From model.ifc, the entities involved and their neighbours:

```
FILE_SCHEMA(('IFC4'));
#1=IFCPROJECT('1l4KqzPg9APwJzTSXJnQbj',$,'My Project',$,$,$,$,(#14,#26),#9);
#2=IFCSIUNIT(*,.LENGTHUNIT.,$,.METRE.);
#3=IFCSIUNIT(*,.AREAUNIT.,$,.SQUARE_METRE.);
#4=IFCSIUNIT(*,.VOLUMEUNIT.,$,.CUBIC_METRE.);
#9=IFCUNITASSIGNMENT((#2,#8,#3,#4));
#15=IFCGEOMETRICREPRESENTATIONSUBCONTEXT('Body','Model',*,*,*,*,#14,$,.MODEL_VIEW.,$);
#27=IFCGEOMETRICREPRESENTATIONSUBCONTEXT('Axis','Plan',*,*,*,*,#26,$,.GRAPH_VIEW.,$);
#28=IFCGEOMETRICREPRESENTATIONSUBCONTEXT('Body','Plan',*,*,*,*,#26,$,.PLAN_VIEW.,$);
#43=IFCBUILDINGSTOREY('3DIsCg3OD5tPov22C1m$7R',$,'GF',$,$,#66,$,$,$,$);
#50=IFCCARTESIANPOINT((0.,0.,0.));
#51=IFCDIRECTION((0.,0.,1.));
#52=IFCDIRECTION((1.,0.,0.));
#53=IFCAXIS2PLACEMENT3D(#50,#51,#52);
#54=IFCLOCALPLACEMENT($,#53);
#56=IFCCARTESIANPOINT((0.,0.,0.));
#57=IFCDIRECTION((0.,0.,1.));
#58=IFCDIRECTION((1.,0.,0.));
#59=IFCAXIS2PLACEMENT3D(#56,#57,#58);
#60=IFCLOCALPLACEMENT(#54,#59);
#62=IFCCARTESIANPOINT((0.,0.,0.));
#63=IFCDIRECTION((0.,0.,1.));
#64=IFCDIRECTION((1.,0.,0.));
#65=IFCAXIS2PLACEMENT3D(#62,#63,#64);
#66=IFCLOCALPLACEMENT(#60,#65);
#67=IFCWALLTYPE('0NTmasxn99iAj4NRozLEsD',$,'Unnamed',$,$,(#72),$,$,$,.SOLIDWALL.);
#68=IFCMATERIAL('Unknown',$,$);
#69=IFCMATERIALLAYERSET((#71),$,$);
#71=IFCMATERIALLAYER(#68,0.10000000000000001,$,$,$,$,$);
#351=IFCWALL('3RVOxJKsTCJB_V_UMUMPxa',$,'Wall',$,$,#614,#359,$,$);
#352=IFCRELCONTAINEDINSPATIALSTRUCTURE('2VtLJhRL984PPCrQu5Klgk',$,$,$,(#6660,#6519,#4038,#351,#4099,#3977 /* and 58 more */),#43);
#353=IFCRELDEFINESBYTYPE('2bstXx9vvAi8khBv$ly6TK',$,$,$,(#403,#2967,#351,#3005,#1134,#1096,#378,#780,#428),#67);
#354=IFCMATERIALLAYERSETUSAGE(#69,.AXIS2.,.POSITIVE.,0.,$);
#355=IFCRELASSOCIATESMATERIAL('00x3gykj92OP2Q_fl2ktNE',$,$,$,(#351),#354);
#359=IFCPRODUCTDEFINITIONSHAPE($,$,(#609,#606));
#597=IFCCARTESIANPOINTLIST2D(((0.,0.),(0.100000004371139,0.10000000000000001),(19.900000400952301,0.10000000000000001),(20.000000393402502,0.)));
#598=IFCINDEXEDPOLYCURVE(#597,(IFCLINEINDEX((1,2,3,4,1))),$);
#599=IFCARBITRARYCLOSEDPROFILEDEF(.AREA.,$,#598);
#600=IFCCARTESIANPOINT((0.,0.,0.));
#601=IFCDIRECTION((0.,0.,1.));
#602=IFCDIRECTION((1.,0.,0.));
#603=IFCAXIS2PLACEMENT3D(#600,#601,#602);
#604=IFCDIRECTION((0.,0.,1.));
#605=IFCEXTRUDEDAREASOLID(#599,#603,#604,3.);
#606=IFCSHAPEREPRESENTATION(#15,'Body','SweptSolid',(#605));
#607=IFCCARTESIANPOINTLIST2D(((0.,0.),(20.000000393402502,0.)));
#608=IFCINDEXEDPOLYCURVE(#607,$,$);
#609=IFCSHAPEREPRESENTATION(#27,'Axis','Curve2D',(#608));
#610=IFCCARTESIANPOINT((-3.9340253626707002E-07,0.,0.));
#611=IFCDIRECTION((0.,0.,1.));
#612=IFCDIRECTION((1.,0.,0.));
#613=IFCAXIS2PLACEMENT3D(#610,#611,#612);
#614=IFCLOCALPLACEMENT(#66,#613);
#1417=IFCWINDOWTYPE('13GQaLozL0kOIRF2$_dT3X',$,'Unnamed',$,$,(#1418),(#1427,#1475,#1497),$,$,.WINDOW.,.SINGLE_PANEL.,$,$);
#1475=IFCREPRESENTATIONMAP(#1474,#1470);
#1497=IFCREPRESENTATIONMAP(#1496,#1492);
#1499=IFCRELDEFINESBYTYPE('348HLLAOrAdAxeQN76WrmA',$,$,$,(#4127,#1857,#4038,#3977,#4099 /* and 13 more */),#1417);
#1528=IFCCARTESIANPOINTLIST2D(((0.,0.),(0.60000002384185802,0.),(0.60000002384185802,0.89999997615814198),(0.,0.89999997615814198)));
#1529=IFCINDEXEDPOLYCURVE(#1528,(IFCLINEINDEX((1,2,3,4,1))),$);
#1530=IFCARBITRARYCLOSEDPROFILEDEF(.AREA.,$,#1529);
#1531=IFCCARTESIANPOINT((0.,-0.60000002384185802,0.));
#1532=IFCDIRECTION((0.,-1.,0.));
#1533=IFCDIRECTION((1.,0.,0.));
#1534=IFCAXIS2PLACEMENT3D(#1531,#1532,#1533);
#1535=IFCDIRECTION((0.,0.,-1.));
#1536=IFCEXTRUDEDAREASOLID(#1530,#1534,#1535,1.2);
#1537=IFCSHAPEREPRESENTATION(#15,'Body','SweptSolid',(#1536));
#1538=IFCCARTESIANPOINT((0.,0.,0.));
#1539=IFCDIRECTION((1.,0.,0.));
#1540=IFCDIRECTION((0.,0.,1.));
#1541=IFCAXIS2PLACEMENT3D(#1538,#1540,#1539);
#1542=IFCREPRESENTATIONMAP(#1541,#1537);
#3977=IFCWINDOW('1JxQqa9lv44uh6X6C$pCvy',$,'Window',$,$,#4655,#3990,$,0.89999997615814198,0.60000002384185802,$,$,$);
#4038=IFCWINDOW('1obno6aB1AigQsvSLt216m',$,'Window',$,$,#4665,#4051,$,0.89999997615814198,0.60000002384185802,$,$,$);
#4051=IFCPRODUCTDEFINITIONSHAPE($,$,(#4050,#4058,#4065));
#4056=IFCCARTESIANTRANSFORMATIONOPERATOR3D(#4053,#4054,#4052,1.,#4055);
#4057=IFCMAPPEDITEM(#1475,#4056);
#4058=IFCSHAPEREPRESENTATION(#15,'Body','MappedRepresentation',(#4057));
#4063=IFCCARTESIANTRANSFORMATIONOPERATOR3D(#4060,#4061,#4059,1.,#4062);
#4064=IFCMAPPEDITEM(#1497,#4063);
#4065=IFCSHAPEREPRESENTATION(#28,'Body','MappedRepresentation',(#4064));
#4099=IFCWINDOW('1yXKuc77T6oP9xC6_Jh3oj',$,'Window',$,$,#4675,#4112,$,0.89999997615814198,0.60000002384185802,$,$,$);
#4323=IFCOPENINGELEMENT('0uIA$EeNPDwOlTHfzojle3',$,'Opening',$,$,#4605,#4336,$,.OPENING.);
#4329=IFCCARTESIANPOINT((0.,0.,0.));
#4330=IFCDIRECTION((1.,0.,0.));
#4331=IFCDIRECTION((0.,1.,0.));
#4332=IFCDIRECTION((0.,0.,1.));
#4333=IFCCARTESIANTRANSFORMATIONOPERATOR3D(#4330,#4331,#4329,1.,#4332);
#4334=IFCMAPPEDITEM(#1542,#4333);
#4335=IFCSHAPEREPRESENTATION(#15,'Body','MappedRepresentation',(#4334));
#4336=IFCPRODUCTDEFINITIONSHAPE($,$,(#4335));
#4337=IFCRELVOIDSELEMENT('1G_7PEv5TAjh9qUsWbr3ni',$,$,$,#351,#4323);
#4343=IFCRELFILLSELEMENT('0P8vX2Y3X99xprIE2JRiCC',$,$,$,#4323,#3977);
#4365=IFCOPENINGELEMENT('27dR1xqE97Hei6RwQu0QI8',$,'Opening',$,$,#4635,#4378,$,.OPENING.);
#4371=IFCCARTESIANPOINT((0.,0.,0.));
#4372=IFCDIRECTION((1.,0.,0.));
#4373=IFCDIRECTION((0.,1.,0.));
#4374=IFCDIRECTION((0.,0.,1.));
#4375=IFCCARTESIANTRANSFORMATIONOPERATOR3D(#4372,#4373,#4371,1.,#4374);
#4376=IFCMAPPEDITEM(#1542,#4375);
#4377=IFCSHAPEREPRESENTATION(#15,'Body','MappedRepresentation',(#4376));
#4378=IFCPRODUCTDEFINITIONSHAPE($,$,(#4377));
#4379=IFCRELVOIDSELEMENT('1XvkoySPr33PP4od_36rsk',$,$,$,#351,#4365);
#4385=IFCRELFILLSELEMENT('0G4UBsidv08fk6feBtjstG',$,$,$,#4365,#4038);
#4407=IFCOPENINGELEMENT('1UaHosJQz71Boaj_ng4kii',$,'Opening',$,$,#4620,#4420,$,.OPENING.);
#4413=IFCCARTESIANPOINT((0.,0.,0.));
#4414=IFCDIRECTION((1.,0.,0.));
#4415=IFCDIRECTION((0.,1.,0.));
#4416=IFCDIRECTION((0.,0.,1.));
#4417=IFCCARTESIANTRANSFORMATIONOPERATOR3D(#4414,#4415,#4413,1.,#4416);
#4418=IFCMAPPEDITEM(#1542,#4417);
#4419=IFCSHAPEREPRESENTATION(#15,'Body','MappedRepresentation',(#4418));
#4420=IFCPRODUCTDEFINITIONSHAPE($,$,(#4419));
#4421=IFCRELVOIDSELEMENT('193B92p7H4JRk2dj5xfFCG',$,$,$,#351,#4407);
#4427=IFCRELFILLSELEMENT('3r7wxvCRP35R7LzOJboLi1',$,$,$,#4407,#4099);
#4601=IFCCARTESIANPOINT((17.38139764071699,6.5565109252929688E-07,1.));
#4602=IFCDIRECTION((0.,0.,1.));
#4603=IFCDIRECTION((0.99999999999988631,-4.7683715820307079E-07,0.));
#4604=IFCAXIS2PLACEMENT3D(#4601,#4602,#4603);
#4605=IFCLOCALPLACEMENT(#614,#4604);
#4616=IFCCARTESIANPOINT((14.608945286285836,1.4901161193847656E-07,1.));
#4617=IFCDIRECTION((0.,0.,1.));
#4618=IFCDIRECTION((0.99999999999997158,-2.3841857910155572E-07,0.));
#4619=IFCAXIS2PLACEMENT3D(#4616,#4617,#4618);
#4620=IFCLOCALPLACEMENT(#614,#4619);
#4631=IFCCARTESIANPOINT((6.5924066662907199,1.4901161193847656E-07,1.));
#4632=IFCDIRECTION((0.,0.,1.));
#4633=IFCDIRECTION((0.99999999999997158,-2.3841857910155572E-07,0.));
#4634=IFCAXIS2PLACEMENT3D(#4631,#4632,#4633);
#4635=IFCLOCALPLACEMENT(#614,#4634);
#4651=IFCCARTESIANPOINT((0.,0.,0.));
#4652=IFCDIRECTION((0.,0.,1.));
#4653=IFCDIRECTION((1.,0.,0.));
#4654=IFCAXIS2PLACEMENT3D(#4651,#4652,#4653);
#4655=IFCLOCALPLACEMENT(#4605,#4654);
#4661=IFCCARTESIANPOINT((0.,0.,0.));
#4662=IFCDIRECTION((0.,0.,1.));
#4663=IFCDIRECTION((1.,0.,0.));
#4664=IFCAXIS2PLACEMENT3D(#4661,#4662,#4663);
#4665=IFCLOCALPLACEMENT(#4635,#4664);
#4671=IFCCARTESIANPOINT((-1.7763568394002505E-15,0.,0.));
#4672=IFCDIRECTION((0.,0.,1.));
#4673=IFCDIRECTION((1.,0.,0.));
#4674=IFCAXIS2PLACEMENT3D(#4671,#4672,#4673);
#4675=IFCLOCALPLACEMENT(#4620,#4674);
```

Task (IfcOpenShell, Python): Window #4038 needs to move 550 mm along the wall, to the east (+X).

```python
import ifcopenshell
import ifcopenshell.api.geometry
import ifcopenshell.util.placement
import ifcopenshell.util.unit

model = ifcopenshell.open("model.ifc")
unit_scale = ifcopenshell.util.unit.calculate_unit_scale(model)

window = model.by_guid("1obno6aB1AigQsvSLt216m")
opening = window.FillsVoids[0].RelatingOpeningElement
wall = opening.VoidsElements[0].RelatingBuildingElement

wall_matrix = ifcopenshell.util.placement.get_local_placement(wall.ObjectPlacement)
shift = wall_matrix[:3, 0] * 0.55 / unit_scale
before = ifcopenshell.util.placement.get_local_placement(window.ObjectPlacement)[:3, 3].copy()

# The window is placed relative to its opening, so it follows when the opening moves.
matrix = ifcopenshell.util.placement.get_local_placement(opening.ObjectPlacement)
matrix[:3, 3] += shift
ifcopenshell.api.geometry.edit_object_placement(
    model, product=opening, matrix=matrix, is_si=False, should_transform_children=True
)

after = ifcopenshell.util.placement.get_local_placement(window.ObjectPlacement)[:3, 3]
print("window moved by", (after - before).round(3) + 0.0)

model.write("model_rev.ifc")
```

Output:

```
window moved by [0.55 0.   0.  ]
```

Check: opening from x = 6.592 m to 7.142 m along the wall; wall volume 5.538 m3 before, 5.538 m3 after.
